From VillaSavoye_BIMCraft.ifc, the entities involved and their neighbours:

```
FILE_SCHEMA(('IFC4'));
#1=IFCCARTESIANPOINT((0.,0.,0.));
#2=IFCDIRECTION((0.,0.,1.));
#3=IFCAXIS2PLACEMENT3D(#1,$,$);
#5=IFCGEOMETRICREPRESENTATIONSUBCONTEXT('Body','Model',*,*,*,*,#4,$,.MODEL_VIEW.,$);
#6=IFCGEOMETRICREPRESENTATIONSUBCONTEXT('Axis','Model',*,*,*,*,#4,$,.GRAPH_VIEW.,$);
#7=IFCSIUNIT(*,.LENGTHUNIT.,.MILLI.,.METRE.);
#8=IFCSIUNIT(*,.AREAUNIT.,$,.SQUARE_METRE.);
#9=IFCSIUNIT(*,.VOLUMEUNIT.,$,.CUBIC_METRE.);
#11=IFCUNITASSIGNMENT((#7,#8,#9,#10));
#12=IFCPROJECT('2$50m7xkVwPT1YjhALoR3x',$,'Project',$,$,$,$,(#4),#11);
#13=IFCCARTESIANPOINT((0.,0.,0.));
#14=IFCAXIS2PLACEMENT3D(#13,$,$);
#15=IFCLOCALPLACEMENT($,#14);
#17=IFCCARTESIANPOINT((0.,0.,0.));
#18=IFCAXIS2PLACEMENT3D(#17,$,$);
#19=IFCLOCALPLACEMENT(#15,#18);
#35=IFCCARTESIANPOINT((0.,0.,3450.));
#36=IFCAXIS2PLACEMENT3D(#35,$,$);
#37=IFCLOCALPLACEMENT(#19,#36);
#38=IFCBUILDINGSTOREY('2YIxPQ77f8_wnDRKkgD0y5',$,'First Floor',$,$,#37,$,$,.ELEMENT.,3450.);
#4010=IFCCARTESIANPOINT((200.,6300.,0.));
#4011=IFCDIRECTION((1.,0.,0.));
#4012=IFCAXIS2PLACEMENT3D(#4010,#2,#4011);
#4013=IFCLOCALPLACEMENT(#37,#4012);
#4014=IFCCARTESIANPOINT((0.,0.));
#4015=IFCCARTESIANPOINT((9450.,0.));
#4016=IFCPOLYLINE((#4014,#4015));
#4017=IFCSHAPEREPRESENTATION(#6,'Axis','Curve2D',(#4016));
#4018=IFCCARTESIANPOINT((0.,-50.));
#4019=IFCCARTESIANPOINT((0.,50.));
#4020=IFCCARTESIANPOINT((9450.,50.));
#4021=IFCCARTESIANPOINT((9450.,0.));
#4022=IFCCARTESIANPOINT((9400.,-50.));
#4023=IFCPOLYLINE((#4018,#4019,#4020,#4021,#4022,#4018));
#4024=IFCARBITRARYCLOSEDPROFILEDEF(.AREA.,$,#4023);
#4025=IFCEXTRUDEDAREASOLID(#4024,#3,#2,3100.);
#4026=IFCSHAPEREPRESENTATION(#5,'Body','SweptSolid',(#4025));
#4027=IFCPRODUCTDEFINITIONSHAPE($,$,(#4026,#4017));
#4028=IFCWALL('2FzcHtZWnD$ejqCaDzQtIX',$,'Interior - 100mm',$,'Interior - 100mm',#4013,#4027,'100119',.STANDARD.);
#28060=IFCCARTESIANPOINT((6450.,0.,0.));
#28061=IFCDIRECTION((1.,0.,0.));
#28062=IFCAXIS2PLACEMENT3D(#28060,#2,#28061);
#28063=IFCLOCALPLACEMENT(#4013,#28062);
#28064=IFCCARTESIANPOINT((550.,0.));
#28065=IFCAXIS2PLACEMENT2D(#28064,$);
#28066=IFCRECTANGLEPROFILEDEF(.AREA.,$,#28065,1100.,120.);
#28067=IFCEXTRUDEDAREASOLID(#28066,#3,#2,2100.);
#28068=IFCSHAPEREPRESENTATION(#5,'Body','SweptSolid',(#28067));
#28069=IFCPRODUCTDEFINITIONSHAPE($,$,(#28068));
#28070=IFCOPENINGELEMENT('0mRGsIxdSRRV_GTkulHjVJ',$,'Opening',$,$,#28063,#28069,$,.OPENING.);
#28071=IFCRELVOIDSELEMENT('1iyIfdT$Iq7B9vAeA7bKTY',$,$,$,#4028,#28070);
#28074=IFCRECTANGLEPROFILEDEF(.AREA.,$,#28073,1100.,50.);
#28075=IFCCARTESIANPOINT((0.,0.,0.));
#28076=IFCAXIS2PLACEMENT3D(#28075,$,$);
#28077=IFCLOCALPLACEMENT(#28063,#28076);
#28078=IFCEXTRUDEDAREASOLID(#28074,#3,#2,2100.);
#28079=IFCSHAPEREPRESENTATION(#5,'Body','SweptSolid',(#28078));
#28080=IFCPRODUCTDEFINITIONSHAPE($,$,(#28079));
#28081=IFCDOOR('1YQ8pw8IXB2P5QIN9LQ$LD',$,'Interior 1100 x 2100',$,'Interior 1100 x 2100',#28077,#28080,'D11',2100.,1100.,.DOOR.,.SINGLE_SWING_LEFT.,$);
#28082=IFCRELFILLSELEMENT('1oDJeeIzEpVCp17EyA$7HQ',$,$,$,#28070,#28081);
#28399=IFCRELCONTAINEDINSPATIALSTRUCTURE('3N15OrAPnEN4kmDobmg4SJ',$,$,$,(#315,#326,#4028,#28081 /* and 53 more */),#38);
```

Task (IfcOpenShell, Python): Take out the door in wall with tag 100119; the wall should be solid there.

```python
import ifcopenshell
import ifcopenshell.api.feature
import ifcopenshell.api.root
import ifcopenshell.geom
import ifcopenshell.util.shape

model = ifcopenshell.open("VillaSavoye_BIMCraft.ifc")
settings = ifcopenshell.geom.settings()


def volume(element):
    """Net volume in cubic metres, openings subtracted."""
    shape = ifcopenshell.geom.create_shape(settings, element)
    return ifcopenshell.util.shape.get_volume(shape.geometry)


door = model.by_guid("1YQ8pw8IXB2P5QIN9LQ$LD")
opening = door.FillsVoids[0].RelatingOpeningElement
wall = opening.VoidsElements[0].RelatingBuildingElement
before = volume(wall)

ifcopenshell.api.root.remove_product(model, product=door)
ifcopenshell.api.feature.remove_feature(model, feature=opening)

after = volume(wall)

print(f"wall volume {before:.3f} -> {after:.3f} m3")

model.write("VillaSavoye_BIMCraft_rev.ifc")
```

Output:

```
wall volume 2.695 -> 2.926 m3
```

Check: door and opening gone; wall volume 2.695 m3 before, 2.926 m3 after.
